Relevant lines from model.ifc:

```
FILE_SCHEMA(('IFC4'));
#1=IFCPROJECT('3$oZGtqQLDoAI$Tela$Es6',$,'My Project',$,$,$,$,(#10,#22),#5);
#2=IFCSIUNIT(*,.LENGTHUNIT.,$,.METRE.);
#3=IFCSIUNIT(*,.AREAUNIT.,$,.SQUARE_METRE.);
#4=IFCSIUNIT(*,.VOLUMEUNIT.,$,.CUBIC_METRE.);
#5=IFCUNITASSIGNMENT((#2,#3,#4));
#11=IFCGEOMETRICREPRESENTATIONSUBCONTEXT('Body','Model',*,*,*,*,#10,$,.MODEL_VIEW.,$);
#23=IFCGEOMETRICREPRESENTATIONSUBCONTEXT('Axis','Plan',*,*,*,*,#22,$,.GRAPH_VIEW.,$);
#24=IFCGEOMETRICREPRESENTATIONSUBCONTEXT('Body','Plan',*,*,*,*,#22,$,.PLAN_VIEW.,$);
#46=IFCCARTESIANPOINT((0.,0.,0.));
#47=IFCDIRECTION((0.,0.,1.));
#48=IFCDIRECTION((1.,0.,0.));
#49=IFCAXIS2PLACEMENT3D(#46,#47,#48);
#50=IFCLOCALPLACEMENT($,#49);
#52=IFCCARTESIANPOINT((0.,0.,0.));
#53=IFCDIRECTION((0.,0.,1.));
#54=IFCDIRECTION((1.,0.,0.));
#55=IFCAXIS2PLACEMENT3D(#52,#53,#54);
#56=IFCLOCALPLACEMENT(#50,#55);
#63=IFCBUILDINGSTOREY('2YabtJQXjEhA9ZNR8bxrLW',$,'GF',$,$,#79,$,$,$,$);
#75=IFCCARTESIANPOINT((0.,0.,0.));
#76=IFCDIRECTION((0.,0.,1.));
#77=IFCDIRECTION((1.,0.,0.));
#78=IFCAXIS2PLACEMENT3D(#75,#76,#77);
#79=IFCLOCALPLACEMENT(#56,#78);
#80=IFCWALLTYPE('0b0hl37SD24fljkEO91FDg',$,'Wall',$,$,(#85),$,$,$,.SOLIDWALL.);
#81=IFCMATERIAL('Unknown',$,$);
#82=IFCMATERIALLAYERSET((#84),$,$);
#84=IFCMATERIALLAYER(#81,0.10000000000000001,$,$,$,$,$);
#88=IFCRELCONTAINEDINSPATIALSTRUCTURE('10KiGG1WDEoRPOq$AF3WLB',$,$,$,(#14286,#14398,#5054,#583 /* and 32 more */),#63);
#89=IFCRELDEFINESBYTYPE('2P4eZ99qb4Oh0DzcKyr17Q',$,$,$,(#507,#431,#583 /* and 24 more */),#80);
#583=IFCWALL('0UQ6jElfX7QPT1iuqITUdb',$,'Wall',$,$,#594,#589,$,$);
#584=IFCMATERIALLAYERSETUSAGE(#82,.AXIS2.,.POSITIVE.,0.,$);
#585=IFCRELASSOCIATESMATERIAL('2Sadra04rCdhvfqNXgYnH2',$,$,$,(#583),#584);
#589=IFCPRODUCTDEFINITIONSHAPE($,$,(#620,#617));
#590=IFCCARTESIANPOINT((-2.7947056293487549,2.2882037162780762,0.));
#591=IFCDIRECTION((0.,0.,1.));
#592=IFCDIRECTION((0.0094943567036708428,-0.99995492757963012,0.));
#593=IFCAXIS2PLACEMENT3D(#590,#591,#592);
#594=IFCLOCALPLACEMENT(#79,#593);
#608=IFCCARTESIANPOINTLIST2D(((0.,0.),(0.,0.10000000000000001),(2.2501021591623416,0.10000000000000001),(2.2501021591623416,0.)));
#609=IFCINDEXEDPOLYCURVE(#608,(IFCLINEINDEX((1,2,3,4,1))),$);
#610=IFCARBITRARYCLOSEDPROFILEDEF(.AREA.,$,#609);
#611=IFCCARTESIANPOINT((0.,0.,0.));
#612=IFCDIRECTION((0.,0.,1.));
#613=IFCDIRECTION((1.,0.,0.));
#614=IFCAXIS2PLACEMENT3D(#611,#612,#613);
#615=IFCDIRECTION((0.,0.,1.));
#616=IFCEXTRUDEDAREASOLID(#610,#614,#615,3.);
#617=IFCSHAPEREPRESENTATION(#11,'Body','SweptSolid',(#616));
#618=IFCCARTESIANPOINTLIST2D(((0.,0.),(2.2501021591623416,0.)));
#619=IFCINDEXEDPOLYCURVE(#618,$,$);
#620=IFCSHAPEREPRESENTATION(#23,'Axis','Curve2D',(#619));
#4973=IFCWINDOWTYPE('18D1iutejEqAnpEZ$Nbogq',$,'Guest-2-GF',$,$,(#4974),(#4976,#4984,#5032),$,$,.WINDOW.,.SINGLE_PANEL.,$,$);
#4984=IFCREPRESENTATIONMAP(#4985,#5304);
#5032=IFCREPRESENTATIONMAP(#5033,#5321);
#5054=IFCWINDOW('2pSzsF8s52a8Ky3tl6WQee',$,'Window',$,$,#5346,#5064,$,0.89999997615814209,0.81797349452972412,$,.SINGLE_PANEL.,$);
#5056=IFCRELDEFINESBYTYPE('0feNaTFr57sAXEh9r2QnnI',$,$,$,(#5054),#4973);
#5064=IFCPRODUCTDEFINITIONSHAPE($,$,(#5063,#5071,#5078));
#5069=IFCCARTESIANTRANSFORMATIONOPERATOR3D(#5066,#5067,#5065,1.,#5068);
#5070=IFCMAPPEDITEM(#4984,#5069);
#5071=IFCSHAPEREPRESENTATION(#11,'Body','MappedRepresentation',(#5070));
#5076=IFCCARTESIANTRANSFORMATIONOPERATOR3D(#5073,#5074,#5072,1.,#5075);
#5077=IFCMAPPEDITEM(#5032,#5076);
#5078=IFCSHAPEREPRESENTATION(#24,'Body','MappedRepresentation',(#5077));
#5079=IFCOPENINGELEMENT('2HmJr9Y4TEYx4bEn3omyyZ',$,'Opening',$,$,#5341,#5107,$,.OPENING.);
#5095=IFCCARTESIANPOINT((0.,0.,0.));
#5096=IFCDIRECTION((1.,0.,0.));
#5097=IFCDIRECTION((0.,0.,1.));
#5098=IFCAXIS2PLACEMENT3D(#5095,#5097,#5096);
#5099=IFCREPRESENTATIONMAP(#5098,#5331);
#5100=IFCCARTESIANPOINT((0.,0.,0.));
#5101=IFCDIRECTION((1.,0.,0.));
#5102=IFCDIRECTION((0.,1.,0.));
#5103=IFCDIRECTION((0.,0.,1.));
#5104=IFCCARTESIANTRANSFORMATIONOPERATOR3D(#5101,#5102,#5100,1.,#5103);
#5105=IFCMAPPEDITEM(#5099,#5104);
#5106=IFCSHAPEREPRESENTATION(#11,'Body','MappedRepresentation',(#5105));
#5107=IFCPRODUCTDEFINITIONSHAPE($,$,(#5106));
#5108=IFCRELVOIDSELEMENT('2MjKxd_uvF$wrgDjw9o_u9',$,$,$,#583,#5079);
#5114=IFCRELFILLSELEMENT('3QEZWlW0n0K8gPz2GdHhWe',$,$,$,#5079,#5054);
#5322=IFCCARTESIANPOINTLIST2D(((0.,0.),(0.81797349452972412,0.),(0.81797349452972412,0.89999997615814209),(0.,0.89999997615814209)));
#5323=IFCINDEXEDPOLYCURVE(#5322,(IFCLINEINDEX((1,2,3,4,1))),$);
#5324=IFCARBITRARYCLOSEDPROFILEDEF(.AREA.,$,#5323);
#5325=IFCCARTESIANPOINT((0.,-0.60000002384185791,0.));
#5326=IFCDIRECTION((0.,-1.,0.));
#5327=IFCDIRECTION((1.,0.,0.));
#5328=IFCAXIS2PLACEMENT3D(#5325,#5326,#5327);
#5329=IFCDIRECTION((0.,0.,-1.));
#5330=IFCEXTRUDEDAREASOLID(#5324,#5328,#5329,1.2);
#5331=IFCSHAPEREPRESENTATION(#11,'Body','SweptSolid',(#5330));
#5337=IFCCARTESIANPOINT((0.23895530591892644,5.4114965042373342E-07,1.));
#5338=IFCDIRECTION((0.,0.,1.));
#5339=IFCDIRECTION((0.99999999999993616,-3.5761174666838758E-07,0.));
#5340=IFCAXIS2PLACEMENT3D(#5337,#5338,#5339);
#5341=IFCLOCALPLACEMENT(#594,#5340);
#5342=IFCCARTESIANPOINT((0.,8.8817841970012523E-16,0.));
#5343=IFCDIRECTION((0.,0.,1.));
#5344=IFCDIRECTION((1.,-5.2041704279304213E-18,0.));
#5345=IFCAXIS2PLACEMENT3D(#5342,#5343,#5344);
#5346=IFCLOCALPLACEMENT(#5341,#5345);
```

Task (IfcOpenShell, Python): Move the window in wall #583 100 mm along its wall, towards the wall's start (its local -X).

```python
import ifcopenshell
import ifcopenshell.api.geometry
import ifcopenshell.util.placement
import ifcopenshell.util.unit

model = ifcopenshell.open("model.ifc")
unit_scale = ifcopenshell.util.unit.calculate_unit_scale(model)

window = model.by_guid("2pSzsF8s52a8Ky3tl6WQee")
opening = window.FillsVoids[0].RelatingOpeningElement
wall = opening.VoidsElements[0].RelatingBuildingElement

wall_matrix = ifcopenshell.util.placement.get_local_placement(wall.ObjectPlacement)
shift = wall_matrix[:3, 0] * -0.1 / unit_scale
before = ifcopenshell.util.placement.get_local_placement(window.ObjectPlacement)[:3, 3].copy()

# The window is placed relative to its opening, so it follows when the opening moves.
matrix = ifcopenshell.util.placement.get_local_placement(opening.ObjectPlacement)
matrix[:3, 3] += shift
ifcopenshell.api.geometry.edit_object_placement(
    model, product=opening, matrix=matrix, is_si=False, should_transform_children=True
)

after = ifcopenshell.util.placement.get_local_placement(window.ObjectPlacement)[:3, 3]
print("window moved by", (after - before).round(3) + 0.0)

model.write("model_edited.ifc")
```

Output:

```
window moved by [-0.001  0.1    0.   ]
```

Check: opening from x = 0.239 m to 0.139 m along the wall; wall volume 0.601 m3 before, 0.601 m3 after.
